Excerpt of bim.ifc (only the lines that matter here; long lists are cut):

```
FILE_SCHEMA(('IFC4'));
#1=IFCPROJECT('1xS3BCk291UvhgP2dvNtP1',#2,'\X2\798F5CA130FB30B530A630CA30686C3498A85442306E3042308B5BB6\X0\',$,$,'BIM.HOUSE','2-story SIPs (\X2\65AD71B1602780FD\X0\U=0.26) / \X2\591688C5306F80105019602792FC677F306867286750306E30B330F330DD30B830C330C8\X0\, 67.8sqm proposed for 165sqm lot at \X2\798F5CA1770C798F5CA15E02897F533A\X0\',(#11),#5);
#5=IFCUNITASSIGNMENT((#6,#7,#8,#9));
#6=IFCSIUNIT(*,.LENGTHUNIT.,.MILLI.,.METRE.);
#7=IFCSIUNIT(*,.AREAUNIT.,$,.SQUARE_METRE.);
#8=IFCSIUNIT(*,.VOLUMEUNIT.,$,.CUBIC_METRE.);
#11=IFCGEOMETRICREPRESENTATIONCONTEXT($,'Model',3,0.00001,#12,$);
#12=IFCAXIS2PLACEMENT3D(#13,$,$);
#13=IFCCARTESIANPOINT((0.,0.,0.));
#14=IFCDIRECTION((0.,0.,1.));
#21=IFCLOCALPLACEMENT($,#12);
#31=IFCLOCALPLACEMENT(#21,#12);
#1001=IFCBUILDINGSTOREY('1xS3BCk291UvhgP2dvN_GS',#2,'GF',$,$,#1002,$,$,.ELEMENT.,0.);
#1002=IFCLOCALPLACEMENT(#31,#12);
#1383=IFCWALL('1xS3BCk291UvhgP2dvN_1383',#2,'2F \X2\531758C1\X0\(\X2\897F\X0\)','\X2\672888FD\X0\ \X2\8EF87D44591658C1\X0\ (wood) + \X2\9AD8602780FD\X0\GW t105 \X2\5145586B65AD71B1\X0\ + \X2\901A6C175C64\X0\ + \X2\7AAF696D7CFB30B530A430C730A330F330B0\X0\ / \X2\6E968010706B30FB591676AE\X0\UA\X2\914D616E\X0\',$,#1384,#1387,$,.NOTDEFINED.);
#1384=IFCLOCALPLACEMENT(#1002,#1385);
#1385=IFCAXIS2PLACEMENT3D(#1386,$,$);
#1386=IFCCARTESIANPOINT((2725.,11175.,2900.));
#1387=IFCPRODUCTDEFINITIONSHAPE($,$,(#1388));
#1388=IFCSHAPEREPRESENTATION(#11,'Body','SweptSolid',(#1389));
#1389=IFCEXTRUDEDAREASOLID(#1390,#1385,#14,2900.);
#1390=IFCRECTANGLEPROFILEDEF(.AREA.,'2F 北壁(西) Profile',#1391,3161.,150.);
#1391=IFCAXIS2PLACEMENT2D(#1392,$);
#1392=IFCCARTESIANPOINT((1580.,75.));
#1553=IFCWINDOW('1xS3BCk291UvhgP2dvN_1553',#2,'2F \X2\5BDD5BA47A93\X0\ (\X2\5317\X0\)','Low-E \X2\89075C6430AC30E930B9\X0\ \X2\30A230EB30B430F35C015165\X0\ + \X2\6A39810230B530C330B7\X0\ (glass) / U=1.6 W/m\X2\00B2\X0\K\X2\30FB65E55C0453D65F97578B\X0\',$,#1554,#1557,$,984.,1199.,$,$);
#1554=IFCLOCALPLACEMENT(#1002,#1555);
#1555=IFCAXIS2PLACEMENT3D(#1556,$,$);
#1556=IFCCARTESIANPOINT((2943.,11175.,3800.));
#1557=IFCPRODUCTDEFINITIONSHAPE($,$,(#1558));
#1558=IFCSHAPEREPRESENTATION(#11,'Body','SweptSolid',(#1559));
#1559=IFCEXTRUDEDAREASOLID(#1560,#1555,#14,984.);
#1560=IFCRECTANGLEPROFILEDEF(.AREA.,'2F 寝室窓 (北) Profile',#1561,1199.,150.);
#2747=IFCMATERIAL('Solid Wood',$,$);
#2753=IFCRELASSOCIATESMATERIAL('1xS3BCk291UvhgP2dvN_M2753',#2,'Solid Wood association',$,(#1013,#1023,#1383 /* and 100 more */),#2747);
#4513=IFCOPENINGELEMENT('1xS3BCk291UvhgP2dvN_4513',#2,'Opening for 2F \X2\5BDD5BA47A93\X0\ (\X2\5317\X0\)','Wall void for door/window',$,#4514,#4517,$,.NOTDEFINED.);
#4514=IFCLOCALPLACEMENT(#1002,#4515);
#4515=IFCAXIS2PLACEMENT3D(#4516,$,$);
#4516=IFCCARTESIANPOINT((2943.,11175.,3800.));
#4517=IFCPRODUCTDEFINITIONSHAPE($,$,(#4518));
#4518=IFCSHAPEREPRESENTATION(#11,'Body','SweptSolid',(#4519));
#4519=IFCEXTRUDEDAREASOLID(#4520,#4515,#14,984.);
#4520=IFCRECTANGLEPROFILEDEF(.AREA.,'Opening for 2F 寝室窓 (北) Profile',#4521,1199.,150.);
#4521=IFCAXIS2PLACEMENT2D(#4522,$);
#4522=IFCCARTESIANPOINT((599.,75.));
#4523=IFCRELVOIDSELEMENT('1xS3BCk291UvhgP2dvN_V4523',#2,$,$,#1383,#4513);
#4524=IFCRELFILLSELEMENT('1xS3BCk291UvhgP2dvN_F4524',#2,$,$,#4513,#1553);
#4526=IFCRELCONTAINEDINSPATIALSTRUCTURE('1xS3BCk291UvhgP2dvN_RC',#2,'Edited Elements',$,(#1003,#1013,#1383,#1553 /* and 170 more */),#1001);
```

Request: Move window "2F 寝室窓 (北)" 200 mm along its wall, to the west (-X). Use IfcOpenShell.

```python
import ifcopenshell
import ifcopenshell.api.geometry
import ifcopenshell.util.placement
import ifcopenshell.util.unit

model = ifcopenshell.open("bim.ifc")
unit_scale = ifcopenshell.util.unit.calculate_unit_scale(model)

window = model.by_id(1553)
opening = window.FillsVoids[0].RelatingOpeningElement
wall = opening.VoidsElements[0].RelatingBuildingElement

wall_matrix = ifcopenshell.util.placement.get_local_placement(wall.ObjectPlacement)
shift = wall_matrix[:3, 0] * -0.2 / unit_scale
before = ifcopenshell.util.placement.get_local_placement(window.ObjectPlacement)[:3, 3].copy()

# The window is not placed relative to its opening, so move both.
for product in (opening, window):
    matrix = ifcopenshell.util.placement.get_local_placement(product.ObjectPlacement)
    matrix[:3, 3] += shift
    ifcopenshell.api.geometry.edit_object_placement(model, product=product, matrix=matrix, is_si=False)

after = ifcopenshell.util.placement.get_local_placement(window.ObjectPlacement)[:3, 3]
print("window moved by", (after - before).round(3) + 0.0)

model.write("bim_v2.ifc")
```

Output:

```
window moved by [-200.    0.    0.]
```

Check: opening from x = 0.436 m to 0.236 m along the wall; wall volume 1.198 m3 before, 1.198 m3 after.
